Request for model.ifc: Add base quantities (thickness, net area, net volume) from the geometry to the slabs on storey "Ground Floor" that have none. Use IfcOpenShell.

First a look at what the model holds.

```python
import ifcopenshell
import ifcopenshell.util.element
import ifcopenshell.util.unit

model = ifcopenshell.open("model.ifc")
print(model.schema)
for unit_type in ("LENGTHUNIT", "AREAUNIT", "VOLUMEUNIT"):
    print(unit_type, ifcopenshell.util.unit.calculate_unit_scale(model, unit_type))
storey = next(s for s in model.by_type("IfcBuildingStorey") if s.Name == "Ground Floor")
slabs = [e for e in ifcopenshell.util.element.get_decomposition(storey) if e.is_a("IfcSlab")]
for e in sorted(slabs, key=lambda e: e.id()):
    print(e.id(), e.is_a(), e.Name, list(ifcopenshell.util.element.get_psets(e, qtos_only=True)), sep=" | ")
```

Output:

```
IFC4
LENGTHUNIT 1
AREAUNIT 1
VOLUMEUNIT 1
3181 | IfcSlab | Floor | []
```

```python
import ifcopenshell
import ifcopenshell.api.pset
import ifcopenshell.geom
import ifcopenshell.util.element
import ifcopenshell.util.shape
import ifcopenshell.util.unit

model = ifcopenshell.open("model.ifc")
unit_scale = ifcopenshell.util.unit.calculate_unit_scale(model)
area_scale = ifcopenshell.util.unit.calculate_unit_scale(model, "AREAUNIT")
volume_scale = ifcopenshell.util.unit.calculate_unit_scale(model, "VOLUMEUNIT")
settings = ifcopenshell.geom.settings()

storey = next(s for s in model.by_type("IfcBuildingStorey") if s.Name == "Ground Floor")
slabs = [e for e in ifcopenshell.util.element.get_decomposition(storey) if e.is_a("IfcSlab")]

for e in sorted(slabs, key=lambda e: e.id()):
    if ifcopenshell.util.element.get_psets(e, qtos_only=True, should_inherit=False):
        continue
    # Geometry comes back in metres, in the element's own axes.
    shape = ifcopenshell.geom.create_shape(settings, e)
    values = {
        "Width": ifcopenshell.util.shape.get_z(shape.geometry) / unit_scale,
        "NetArea": ifcopenshell.util.shape.get_footprint_area(shape.geometry) / area_scale,
        "NetVolume": ifcopenshell.util.shape.get_volume(shape.geometry) / volume_scale,
    }
    qto = ifcopenshell.api.pset.add_qto(model, product=e, name="Qto_SlabBaseQuantities")
    ifcopenshell.api.pset.edit_qto(model, qto=qto, properties=values)
    print(e.id(), {k: round(v, 3) for k, v in values.items()})

model.write("model_rev.ifc")
```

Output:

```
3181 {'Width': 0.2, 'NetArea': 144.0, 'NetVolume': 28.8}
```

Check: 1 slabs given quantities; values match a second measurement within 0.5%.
